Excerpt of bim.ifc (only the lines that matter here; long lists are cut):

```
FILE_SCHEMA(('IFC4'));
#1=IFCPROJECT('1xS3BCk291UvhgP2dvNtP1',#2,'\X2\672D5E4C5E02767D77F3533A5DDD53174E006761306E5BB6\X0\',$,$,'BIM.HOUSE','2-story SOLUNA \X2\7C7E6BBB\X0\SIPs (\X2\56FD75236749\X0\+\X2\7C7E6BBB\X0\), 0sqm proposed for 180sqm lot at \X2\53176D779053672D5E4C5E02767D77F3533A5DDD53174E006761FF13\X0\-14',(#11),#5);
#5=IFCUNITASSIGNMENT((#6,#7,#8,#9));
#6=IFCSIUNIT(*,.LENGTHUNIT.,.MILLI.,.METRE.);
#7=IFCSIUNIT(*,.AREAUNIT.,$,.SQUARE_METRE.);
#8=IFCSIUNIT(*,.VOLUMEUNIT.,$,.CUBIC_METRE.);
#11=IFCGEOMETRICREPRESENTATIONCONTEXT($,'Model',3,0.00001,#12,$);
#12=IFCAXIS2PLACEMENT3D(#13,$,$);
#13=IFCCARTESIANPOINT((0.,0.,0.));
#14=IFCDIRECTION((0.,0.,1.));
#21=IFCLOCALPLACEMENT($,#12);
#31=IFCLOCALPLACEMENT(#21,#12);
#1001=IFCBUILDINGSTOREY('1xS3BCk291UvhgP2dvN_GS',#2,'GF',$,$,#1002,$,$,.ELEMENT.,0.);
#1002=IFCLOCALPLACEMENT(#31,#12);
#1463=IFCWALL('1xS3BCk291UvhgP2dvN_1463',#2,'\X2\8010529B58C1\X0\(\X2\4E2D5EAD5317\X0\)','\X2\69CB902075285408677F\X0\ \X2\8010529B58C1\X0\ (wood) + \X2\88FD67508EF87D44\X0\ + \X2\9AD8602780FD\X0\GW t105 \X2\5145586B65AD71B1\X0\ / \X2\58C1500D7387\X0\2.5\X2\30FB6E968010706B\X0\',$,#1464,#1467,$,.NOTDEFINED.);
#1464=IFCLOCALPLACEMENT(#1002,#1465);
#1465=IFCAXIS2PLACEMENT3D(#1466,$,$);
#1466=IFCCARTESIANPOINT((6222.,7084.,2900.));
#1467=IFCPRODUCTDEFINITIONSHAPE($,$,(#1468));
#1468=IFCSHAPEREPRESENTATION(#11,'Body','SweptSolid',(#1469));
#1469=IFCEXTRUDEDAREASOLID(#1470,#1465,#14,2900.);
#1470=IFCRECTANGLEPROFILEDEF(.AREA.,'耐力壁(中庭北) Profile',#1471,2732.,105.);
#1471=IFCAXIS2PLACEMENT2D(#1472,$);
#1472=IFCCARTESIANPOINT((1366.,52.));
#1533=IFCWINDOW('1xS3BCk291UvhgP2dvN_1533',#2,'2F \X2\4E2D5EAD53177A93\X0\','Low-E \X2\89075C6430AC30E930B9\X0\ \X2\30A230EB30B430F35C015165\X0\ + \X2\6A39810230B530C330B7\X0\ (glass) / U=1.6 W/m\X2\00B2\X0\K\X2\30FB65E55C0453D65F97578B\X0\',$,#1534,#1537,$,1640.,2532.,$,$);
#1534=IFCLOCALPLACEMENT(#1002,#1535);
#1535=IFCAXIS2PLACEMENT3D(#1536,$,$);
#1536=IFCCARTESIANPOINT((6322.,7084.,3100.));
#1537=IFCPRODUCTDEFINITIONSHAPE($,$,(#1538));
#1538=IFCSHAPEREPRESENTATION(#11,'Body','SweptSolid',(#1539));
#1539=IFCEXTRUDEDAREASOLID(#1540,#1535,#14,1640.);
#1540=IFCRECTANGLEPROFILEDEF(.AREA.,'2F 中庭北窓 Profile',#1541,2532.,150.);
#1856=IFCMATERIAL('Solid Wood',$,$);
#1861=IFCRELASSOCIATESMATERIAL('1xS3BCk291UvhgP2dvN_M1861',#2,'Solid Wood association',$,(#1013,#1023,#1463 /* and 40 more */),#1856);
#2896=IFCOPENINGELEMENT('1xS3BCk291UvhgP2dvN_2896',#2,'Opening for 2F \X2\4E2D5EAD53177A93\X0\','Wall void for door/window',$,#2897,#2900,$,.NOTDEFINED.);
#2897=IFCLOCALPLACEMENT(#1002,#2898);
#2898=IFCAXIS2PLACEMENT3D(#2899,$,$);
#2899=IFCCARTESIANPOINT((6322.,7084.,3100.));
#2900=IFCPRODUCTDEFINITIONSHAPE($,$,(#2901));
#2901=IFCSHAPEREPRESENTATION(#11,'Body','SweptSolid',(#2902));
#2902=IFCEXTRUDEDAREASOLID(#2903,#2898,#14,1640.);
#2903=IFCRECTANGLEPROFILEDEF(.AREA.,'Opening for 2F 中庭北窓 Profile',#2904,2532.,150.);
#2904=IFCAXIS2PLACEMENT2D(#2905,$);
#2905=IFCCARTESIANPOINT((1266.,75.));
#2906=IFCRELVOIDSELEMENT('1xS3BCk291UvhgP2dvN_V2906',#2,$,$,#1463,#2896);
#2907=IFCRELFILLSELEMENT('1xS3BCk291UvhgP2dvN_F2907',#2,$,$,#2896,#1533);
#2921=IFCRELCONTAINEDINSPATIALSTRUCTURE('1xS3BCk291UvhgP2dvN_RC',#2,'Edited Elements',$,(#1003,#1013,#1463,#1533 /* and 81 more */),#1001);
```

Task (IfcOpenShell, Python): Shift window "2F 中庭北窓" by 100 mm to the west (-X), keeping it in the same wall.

```python
import ifcopenshell
import ifcopenshell.api.geometry
import ifcopenshell.util.placement
import ifcopenshell.util.unit

model = ifcopenshell.open("bim.ifc")
unit_scale = ifcopenshell.util.unit.calculate_unit_scale(model)

window = model.by_guid("1xS3BCk291UvhgP2dvN_1533")
opening = window.FillsVoids[0].RelatingOpeningElement
wall = opening.VoidsElements[0].RelatingBuildingElement

wall_matrix = ifcopenshell.util.placement.get_local_placement(wall.ObjectPlacement)
shift = wall_matrix[:3, 0] * -0.1 / unit_scale
before = ifcopenshell.util.placement.get_local_placement(window.ObjectPlacement)[:3, 3].copy()

# The window is not placed relative to its opening, so move both.
for product in (opening, window):
    matrix = ifcopenshell.util.placement.get_local_placement(product.ObjectPlacement)
    matrix[:3, 3] += shift
    ifcopenshell.api.geometry.edit_object_placement(model, product=product, matrix=matrix, is_si=False)

after = ifcopenshell.util.placement.get_local_placement(window.ObjectPlacement)[:3, 3]
print("window moved by", (after - before).round(3) + 0.0)

model.write("bim_v2.ifc")
```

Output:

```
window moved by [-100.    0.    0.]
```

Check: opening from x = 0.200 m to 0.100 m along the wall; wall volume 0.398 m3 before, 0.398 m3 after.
